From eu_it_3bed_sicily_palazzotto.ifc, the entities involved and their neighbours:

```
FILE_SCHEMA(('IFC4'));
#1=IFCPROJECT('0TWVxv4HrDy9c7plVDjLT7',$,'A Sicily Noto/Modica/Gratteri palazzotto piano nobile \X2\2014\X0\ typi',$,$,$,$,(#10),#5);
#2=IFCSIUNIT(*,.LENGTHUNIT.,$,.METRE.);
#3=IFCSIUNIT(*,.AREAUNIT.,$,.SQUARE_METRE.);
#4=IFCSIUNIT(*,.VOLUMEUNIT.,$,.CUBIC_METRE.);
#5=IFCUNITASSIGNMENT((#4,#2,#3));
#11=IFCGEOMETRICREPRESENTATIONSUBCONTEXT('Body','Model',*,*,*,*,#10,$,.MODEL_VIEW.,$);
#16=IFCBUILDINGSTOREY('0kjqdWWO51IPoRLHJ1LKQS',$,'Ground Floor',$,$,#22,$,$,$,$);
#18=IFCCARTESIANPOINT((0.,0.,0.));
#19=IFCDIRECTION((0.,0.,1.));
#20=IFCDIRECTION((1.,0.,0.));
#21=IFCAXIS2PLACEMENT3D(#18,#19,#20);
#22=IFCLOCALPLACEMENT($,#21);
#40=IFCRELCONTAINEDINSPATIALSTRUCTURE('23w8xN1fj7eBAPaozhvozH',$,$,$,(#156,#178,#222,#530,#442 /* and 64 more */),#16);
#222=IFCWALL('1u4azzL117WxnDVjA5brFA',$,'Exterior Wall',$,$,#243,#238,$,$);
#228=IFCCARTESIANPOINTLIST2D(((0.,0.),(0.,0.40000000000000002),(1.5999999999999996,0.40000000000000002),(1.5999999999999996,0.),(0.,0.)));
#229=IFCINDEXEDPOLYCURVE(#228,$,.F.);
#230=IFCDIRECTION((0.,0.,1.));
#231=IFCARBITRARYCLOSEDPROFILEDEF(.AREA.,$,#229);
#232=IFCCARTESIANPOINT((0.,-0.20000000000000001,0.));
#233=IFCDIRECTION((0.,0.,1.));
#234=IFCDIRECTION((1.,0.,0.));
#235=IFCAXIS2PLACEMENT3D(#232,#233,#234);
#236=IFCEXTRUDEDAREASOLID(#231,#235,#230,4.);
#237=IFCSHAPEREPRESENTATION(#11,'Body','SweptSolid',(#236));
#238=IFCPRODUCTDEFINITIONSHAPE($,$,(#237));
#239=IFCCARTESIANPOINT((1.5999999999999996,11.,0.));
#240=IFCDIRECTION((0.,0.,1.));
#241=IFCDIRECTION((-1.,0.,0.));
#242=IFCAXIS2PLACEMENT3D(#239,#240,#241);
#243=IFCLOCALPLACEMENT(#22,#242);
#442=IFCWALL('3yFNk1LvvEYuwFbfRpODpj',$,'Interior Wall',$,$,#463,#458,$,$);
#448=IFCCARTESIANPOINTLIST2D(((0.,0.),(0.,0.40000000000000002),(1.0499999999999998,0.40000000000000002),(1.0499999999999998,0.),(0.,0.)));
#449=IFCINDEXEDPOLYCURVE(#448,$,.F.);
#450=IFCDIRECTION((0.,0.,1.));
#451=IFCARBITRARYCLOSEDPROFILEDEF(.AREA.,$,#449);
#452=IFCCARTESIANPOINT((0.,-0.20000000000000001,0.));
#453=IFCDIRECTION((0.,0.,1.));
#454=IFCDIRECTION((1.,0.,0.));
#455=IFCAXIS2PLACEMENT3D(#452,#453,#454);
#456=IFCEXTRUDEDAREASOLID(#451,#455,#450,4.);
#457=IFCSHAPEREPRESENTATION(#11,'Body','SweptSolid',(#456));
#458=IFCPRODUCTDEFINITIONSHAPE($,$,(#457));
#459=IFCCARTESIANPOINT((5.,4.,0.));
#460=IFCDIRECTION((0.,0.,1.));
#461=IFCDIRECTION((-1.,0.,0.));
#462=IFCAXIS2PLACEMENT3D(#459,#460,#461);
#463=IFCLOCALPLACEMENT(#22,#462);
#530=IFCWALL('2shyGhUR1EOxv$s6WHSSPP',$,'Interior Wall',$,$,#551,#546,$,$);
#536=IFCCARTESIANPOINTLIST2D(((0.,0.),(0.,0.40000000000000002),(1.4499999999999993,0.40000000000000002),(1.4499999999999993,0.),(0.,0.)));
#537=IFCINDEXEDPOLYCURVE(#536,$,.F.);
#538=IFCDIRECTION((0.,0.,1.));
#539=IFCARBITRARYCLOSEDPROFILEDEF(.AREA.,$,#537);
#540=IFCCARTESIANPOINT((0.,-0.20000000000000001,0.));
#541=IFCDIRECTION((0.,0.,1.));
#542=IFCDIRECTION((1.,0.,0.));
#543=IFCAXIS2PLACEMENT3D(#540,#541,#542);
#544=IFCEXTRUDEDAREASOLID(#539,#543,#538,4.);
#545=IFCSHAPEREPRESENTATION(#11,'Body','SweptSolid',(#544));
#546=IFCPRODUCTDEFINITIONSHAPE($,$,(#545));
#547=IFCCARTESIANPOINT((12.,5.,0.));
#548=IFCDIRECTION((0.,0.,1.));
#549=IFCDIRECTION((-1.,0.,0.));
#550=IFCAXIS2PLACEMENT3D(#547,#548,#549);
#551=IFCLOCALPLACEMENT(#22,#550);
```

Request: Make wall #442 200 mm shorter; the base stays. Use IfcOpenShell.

```python
import ifcopenshell
import ifcopenshell.geom
import ifcopenshell.util.representation
import ifcopenshell.util.shape
import ifcopenshell.util.unit

model = ifcopenshell.open("eu_it_3bed_sicily_palazzotto.ifc")
unit_scale = ifcopenshell.util.unit.calculate_unit_scale(model)
settings = ifcopenshell.geom.settings()


def volume(element):
    """Net volume in cubic metres, openings subtracted."""
    shape = ifcopenshell.geom.create_shape(settings, element)
    return ifcopenshell.util.shape.get_volume(shape.geometry)


wall = model.by_id(442)
before = volume(wall)

body = ifcopenshell.util.representation.get_representation(wall, "Model", "Body")
solid = body.Items[0]
old_height = solid.Depth
solid.Depth -= 0.2 / unit_scale
after = volume(wall)

print(f"height {old_height:g} -> {solid.Depth:g}, volume {before:.3f} -> {after:.3f} m3")

model.write("eu_it_3bed_sicily_palazzotto-out.ifc")
```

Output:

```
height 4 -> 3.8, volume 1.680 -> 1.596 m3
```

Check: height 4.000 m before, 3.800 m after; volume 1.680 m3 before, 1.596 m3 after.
